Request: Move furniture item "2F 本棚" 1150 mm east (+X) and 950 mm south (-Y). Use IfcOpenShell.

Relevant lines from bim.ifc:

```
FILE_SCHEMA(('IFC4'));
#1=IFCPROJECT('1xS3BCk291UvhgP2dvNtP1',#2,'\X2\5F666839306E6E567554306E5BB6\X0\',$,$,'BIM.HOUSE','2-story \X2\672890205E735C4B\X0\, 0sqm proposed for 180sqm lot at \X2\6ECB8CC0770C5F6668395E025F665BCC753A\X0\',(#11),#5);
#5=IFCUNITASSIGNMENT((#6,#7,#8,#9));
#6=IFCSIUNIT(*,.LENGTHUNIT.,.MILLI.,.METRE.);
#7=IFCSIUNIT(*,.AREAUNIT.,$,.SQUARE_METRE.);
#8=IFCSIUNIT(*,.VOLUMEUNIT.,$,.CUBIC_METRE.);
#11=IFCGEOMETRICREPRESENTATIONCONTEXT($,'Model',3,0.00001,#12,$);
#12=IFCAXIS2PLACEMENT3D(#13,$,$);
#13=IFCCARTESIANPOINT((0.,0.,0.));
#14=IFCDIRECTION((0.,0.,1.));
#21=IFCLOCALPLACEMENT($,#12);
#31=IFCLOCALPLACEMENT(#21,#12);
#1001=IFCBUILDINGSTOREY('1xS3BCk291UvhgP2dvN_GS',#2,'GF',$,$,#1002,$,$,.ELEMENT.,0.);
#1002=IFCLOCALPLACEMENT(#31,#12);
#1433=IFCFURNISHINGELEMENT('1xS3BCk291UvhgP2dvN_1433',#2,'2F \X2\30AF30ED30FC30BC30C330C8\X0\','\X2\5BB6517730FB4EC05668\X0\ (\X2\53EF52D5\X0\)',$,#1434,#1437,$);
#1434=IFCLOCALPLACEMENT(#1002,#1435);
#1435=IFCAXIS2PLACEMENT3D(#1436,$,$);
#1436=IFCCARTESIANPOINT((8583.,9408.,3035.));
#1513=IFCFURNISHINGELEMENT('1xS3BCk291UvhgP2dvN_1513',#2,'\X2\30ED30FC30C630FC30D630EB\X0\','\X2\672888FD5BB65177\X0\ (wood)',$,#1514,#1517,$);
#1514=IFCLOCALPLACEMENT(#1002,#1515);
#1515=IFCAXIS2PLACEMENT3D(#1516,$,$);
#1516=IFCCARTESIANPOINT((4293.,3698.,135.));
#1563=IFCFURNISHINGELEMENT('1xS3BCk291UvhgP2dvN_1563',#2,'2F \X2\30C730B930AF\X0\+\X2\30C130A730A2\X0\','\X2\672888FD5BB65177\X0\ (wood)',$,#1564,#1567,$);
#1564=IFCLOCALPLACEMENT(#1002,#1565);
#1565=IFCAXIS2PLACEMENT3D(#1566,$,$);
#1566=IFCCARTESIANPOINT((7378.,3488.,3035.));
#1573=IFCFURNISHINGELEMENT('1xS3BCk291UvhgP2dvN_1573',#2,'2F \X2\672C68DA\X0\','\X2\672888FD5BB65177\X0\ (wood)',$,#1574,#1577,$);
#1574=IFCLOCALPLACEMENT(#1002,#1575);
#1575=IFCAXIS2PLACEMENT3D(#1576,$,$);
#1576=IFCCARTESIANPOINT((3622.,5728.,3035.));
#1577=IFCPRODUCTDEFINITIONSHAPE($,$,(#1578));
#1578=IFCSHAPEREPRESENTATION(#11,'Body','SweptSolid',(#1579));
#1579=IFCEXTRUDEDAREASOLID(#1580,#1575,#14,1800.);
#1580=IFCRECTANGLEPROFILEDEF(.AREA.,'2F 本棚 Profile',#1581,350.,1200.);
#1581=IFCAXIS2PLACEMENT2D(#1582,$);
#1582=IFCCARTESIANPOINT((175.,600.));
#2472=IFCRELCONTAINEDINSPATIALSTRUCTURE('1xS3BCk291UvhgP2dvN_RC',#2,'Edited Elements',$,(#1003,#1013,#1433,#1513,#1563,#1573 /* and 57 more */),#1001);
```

```python
import ifcopenshell
import ifcopenshell.api.geometry
import ifcopenshell.util.placement

model = ifcopenshell.open("bim.ifc")

item = model.by_guid("1xS3BCk291UvhgP2dvN_1573")
matrix = ifcopenshell.util.placement.get_local_placement(item.ObjectPlacement)
matrix[0, 3] += 1150.0
matrix[1, 3] -= 950.0
ifcopenshell.api.geometry.edit_object_placement(model, product=item, matrix=matrix, is_si=False)

print(ifcopenshell.util.placement.get_local_placement(item.ObjectPlacement).round(3) + 0.0)

model.write("bim_updated.ifc")
```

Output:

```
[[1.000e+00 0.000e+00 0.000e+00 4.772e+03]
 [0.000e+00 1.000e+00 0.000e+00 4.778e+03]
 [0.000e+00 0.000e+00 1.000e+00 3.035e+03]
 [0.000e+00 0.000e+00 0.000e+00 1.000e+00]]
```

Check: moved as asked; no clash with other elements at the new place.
